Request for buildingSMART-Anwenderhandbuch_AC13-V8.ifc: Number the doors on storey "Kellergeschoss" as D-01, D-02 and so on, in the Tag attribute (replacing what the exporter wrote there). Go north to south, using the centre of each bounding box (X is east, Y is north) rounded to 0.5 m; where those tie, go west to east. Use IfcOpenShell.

First a look at what the model holds.

```python
import ifcopenshell
import ifcopenshell.util.element
import ifcopenshell.util.placement

model = ifcopenshell.open("buildingSMART-Anwenderhandbuch_AC13-V8.ifc")
print(model.schema)
storey = next(s for s in model.by_type("IfcBuildingStorey") if s.Name == "Kellergeschoss")
doors = [e for e in ifcopenshell.util.element.get_decomposition(storey) if e.is_a("IfcDoor")]
for e in sorted(doors, key=lambda e: e.id()):
    origin = ifcopenshell.util.placement.get_local_placement(e.ObjectPlacement)[:3, 3]
    print(e.id(), e.Tag, e.Name, origin.round(2) + 0.0, sep=" | ")
```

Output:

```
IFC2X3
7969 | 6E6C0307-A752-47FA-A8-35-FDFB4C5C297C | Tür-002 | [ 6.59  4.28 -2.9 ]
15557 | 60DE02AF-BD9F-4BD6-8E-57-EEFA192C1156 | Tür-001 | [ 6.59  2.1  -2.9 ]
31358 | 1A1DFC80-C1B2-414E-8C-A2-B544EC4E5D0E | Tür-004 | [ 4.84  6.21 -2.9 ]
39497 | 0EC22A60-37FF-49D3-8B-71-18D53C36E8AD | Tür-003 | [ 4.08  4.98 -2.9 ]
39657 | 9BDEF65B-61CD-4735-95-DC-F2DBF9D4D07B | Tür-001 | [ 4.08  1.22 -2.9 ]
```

```python
import ifcopenshell
import ifcopenshell.geom
import ifcopenshell.util.element
import ifcopenshell.util.shape

model = ifcopenshell.open("buildingSMART-Anwenderhandbuch_AC13-V8.ifc")
settings = ifcopenshell.geom.settings()
settings.set("use-world-coords", True)


def centre(element):
    shape = ifcopenshell.geom.create_shape(settings, element)
    return ifcopenshell.util.shape.get_bbox_centroid(shape.geometry)


storey = next(s for s in model.by_type("IfcBuildingStorey") if s.Name == "Kellergeschoss")
doors = [e for e in ifcopenshell.util.element.get_decomposition(storey) if e.is_a("IfcDoor")]

# Insertion points can sit at a corner or the storey origin, so sort by the geometry (in metres).
centres = {e: centre(e) for e in doors}
doors.sort(key=lambda e: (-round(centres[e][1] / 0.5), centres[e][0]))

for i, e in enumerate(doors, start=1):
    number = f"D-{i:02d}"
    e.Tag = number
    print(e.id(), number)

model.write("buildingSMART-Anwenderhandbuch_AC13-V8-out.ifc")
```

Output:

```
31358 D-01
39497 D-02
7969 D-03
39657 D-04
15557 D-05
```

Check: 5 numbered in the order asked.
